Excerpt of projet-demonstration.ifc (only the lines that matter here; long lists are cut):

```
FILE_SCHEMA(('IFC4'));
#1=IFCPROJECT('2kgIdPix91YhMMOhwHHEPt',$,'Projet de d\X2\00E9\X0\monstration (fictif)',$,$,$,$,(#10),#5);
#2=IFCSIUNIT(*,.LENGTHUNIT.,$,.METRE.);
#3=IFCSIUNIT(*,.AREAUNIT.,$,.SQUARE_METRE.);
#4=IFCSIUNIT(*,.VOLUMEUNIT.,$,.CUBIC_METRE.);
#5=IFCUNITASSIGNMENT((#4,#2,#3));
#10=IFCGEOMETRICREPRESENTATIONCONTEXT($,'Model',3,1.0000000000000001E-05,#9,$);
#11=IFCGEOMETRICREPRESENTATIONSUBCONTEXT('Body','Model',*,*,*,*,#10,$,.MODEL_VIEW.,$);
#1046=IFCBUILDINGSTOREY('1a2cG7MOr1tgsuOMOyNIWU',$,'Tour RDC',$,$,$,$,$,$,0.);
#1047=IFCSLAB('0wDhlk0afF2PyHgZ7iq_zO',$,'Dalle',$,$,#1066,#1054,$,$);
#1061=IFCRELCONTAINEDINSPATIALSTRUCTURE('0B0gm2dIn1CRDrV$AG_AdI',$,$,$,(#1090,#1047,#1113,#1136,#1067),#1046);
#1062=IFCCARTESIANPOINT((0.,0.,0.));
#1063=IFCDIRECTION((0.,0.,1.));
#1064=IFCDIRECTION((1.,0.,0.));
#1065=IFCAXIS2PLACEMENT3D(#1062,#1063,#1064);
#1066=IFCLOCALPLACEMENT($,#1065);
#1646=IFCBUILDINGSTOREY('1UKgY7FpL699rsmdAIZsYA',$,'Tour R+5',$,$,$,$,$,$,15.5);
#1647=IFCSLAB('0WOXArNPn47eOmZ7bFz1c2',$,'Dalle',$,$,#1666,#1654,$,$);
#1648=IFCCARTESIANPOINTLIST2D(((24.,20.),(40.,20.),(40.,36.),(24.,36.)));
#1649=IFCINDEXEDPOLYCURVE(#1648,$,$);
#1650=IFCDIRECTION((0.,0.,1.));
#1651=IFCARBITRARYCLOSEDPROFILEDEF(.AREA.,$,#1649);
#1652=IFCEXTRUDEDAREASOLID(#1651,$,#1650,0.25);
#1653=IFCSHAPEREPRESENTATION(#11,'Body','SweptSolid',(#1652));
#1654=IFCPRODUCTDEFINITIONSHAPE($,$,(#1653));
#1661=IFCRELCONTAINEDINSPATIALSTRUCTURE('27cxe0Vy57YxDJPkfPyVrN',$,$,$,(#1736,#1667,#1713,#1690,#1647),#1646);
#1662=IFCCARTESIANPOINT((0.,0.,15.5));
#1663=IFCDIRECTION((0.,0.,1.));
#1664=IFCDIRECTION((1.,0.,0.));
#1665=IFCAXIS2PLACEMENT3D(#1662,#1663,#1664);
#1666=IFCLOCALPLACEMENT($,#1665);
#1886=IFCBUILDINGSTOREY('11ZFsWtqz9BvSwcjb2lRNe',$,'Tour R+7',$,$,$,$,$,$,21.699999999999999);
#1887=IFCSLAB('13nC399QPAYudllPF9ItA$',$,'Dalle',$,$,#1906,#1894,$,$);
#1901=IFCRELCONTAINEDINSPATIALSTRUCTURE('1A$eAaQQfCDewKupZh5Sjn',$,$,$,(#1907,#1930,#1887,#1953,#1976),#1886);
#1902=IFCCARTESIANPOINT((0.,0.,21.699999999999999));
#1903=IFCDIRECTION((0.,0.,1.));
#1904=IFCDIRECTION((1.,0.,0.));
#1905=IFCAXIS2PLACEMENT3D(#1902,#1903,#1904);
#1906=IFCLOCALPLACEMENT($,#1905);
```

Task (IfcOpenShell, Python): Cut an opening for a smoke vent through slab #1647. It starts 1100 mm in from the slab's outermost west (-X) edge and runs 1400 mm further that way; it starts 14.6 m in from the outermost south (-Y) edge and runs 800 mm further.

```python
import numpy as np
import ifcopenshell
import ifcopenshell.api.feature
import ifcopenshell.api.geometry
import ifcopenshell.api.root
import ifcopenshell.geom
import ifcopenshell.util.placement
import ifcopenshell.util.representation
import ifcopenshell.util.shape
import ifcopenshell.util.unit

model = ifcopenshell.open("projet-demonstration.ifc")
unit_scale = ifcopenshell.util.unit.calculate_unit_scale(model)
settings = ifcopenshell.geom.settings()


def volume(element):
    """Net volume in cubic metres, openings subtracted."""
    shape = ifcopenshell.geom.create_shape(settings, element)
    return ifcopenshell.util.shape.get_volume(shape.geometry)


slab = model.by_guid("0WOXArNPn47eOmZ7bFz1c2")
before = volume(slab)

# Extent in the slab's own axes, in metres. The edges named are its -X and -Y sides.
slab_shape = ifcopenshell.geom.create_shape(settings, slab)
vertices = ifcopenshell.util.shape.get_vertices(slab_shape.geometry)
x_min, y_min, bottom = vertices.min(axis=0)
top = vertices[:, 2].max()

opening = ifcopenshell.api.root.create_entity(model, ifc_class="IfcOpeningElement", name="Smoke vent opening", predefined_type="OPENING")
context = ifcopenshell.util.representation.get_context(model, "Model", "Body", "MODEL_VIEW")
width, depth = 1.4, 0.8
outline = [(0.0, 0.0), (width, 0.0), (width, depth), (0.0, depth), (0.0, 0.0)]
# Overshoot both faces by 50 mm so the cut is clean.
shape = ifcopenshell.api.geometry.add_slab_representation(
    model, context=context, depth=top - bottom + 0.1, polyline=outline
)
ifcopenshell.api.geometry.assign_representation(model, product=opening, representation=shape)

matrix = ifcopenshell.util.placement.get_local_placement(slab.ObjectPlacement)
matrix[:, 3] = matrix @ np.append(np.array([x_min + 1.1, y_min + 14.6, bottom - 0.05]) / unit_scale, 1.0)
ifcopenshell.api.geometry.edit_object_placement(model, product=opening, matrix=matrix, is_si=False)
ifcopenshell.api.feature.add_feature(model, feature=opening, element=slab)

after = volume(slab)

print(f"slab volume {before:.3f} -> {after:.3f} m3")

model.write("projet-demonstration_updated.ifc")
```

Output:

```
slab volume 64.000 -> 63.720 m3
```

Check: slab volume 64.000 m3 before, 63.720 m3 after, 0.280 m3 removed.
